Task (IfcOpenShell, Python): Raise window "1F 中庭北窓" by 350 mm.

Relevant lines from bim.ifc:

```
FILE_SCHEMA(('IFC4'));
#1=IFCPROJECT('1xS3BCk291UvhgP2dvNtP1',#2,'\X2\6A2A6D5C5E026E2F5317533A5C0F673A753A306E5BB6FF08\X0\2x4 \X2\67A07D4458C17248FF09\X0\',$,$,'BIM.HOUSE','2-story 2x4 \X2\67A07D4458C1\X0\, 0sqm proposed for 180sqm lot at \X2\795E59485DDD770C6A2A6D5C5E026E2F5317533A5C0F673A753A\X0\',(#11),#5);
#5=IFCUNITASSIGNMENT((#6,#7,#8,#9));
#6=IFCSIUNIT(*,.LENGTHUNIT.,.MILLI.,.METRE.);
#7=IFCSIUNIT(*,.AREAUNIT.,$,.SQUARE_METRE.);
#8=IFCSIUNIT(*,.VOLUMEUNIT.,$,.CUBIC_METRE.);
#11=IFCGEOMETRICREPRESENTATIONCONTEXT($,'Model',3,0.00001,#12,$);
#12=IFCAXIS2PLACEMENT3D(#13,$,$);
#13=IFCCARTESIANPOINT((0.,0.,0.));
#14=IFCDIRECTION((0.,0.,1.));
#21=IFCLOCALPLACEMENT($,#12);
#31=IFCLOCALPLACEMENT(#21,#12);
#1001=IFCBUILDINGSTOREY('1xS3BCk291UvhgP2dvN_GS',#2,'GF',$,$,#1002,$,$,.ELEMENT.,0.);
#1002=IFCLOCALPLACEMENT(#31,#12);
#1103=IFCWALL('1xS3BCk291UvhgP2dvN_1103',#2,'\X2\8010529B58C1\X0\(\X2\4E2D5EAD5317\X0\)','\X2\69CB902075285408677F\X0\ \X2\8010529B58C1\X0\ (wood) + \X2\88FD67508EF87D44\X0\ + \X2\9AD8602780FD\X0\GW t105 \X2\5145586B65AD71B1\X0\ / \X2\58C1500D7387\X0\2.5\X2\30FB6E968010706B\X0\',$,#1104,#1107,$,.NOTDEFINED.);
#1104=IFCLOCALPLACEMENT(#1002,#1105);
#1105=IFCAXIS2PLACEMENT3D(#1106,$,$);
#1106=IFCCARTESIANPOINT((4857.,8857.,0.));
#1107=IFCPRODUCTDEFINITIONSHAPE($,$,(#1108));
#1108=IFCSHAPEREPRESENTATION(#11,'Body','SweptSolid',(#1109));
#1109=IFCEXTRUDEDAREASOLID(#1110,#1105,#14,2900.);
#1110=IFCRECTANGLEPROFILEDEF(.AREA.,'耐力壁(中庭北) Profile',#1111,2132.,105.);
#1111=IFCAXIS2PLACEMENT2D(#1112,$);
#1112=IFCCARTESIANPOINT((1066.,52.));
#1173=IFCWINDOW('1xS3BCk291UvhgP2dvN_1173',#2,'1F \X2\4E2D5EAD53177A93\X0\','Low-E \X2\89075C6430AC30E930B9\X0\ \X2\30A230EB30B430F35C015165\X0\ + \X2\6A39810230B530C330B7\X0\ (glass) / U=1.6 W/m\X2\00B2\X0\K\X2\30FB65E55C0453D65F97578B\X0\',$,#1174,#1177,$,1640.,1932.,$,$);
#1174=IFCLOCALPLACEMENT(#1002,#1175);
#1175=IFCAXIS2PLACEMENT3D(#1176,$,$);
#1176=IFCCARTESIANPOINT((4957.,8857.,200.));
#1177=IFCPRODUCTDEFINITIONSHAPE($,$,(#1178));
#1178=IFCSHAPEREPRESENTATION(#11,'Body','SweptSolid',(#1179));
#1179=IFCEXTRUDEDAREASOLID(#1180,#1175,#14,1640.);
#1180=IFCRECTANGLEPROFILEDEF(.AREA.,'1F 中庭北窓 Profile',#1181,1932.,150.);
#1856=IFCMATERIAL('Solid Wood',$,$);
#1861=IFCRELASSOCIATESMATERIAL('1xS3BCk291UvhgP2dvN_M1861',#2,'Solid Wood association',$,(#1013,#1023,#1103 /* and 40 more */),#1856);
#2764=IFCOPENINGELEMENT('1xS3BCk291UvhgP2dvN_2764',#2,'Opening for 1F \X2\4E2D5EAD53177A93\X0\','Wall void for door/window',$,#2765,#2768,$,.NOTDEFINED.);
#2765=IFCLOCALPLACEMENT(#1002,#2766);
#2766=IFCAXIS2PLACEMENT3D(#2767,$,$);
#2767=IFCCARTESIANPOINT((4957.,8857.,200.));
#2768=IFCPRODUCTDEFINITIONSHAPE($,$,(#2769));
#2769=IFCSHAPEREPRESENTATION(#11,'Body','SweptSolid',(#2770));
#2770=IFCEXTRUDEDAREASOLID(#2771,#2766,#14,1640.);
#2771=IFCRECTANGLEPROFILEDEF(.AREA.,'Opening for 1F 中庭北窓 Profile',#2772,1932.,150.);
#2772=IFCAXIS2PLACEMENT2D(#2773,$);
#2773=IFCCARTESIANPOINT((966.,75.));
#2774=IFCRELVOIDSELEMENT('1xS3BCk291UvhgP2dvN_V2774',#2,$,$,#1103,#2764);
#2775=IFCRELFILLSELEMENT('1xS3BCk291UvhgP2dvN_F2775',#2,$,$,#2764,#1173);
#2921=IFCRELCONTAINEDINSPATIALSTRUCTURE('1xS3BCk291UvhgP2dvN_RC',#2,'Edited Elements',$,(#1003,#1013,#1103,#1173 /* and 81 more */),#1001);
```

```python
import numpy as np
import ifcopenshell
import ifcopenshell.api.geometry
import ifcopenshell.util.placement
import ifcopenshell.util.unit

model = ifcopenshell.open("bim.ifc")
unit_scale = ifcopenshell.util.unit.calculate_unit_scale(model)

window = model.by_guid("1xS3BCk291UvhgP2dvN_1173")
opening = window.FillsVoids[0].RelatingOpeningElement
dz = 350.0

shift = np.array([0.0, 0.0, dz])
# The window is not placed relative to its opening, so move both.
for product in (opening, window):
    matrix = ifcopenshell.util.placement.get_local_placement(product.ObjectPlacement)
    matrix[:3, 3] += shift
    ifcopenshell.api.geometry.edit_object_placement(model, product=product, matrix=matrix, is_si=False)

print(f"moved by {dz * unit_scale:+.3f} m")

model.write("bim_rev.ifc")
```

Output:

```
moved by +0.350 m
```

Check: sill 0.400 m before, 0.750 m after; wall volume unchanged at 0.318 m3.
